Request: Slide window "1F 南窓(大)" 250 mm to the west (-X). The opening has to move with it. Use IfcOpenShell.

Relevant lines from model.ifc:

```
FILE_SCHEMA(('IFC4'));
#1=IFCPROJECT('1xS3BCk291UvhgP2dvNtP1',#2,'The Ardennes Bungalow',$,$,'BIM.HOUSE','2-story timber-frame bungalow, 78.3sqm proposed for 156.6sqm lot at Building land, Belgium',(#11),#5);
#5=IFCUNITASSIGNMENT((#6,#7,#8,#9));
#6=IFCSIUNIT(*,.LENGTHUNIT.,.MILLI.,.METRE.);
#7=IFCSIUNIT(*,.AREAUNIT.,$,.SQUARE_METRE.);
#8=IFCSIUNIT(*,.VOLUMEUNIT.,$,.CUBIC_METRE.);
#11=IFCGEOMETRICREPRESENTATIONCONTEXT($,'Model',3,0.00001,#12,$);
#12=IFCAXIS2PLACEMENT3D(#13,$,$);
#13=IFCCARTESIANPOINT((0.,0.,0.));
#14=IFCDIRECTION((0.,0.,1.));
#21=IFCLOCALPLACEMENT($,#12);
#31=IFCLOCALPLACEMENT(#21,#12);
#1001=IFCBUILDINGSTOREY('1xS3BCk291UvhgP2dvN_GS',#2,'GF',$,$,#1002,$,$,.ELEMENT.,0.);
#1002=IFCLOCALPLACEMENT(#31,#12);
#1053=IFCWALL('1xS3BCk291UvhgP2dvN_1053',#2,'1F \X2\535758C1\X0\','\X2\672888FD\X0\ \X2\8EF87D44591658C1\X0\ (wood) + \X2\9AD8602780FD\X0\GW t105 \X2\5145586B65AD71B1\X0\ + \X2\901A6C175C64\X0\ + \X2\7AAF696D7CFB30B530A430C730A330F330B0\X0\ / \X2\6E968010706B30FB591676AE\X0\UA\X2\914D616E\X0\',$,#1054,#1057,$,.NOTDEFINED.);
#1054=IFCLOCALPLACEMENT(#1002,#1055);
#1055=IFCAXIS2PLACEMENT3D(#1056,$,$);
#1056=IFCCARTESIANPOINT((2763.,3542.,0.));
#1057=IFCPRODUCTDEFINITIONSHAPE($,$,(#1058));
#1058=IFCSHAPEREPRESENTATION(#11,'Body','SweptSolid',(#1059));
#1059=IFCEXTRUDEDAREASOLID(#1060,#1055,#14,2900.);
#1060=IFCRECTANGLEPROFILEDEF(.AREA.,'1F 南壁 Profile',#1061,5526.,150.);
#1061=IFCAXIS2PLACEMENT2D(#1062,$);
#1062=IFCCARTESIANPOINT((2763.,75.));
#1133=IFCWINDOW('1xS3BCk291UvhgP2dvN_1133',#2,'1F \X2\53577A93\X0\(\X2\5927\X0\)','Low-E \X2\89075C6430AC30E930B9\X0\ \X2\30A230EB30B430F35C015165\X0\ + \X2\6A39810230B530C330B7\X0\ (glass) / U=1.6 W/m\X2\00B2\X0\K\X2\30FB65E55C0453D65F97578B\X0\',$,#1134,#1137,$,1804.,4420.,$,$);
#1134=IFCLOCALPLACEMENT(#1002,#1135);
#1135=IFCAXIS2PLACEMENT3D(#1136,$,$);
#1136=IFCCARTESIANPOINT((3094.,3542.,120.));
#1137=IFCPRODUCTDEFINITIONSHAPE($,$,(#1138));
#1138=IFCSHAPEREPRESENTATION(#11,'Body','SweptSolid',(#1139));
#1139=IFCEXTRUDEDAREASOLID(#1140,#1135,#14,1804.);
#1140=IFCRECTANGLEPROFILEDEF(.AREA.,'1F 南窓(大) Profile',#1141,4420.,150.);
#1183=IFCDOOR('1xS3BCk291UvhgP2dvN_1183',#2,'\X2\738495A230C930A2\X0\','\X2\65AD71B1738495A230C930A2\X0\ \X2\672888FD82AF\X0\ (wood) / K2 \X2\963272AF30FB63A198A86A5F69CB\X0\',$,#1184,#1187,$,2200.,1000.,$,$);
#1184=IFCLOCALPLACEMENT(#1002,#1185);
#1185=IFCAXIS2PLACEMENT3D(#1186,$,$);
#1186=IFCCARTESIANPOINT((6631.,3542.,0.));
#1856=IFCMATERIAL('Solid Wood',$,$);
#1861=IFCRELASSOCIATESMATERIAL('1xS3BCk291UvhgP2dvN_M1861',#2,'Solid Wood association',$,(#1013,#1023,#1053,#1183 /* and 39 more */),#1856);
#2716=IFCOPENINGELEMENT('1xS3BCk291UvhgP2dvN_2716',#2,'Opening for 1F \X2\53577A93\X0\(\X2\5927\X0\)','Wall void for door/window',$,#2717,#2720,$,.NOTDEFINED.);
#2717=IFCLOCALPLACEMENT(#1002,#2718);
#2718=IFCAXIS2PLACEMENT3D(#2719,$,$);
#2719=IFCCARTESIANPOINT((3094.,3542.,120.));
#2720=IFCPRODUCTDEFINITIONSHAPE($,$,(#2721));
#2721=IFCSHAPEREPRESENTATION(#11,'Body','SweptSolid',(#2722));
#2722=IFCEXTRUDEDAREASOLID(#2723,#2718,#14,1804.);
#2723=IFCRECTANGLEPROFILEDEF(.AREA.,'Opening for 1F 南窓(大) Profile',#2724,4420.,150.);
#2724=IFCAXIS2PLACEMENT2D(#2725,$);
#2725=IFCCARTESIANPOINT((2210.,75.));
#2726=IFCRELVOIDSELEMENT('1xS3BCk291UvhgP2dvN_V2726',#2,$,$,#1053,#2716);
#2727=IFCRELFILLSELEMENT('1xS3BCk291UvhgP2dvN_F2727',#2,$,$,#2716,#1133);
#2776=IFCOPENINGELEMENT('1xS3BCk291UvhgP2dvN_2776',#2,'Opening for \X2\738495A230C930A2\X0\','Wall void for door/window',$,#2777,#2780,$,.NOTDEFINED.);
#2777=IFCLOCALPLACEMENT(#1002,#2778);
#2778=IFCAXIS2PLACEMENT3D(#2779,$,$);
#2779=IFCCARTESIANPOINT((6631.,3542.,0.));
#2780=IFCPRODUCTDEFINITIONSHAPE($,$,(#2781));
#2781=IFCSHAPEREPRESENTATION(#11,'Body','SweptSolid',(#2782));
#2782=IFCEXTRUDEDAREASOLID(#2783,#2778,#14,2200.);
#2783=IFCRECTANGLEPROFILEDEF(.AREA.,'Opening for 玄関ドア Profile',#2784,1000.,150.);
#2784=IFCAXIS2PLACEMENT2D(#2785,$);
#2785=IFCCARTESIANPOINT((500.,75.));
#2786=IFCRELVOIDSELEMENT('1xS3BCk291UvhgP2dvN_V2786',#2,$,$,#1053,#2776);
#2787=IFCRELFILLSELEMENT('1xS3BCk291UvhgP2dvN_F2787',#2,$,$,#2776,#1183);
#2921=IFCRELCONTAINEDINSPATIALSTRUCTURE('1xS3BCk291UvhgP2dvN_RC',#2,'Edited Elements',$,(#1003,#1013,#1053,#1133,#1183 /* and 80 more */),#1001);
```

```python
import ifcopenshell
import ifcopenshell.api.geometry
import ifcopenshell.util.placement

model = ifcopenshell.open("model.ifc")

window = model.by_guid("1xS3BCk291UvhgP2dvN_1133")
opening = window.FillsVoids[0].RelatingOpeningElement
wall = opening.VoidsElements[0].RelatingBuildingElement

wall_matrix = ifcopenshell.util.placement.get_local_placement(wall.ObjectPlacement)
shift = wall_matrix[:3, 0] * -250.0
before = ifcopenshell.util.placement.get_local_placement(window.ObjectPlacement)[:3, 3].copy()

# The window is not placed relative to its opening, so move both.
for product in (opening, window):
    matrix = ifcopenshell.util.placement.get_local_placement(product.ObjectPlacement)
    matrix[:3, 3] += shift
    ifcopenshell.api.geometry.edit_object_placement(model, product=product, matrix=matrix, is_si=False)

after = ifcopenshell.util.placement.get_local_placement(window.ObjectPlacement)[:3, 3]
print("window moved by", (after - before).round(3) + 0.0)

model.write("model_edited.ifc")
```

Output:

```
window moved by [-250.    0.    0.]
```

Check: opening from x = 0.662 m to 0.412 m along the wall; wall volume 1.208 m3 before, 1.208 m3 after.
